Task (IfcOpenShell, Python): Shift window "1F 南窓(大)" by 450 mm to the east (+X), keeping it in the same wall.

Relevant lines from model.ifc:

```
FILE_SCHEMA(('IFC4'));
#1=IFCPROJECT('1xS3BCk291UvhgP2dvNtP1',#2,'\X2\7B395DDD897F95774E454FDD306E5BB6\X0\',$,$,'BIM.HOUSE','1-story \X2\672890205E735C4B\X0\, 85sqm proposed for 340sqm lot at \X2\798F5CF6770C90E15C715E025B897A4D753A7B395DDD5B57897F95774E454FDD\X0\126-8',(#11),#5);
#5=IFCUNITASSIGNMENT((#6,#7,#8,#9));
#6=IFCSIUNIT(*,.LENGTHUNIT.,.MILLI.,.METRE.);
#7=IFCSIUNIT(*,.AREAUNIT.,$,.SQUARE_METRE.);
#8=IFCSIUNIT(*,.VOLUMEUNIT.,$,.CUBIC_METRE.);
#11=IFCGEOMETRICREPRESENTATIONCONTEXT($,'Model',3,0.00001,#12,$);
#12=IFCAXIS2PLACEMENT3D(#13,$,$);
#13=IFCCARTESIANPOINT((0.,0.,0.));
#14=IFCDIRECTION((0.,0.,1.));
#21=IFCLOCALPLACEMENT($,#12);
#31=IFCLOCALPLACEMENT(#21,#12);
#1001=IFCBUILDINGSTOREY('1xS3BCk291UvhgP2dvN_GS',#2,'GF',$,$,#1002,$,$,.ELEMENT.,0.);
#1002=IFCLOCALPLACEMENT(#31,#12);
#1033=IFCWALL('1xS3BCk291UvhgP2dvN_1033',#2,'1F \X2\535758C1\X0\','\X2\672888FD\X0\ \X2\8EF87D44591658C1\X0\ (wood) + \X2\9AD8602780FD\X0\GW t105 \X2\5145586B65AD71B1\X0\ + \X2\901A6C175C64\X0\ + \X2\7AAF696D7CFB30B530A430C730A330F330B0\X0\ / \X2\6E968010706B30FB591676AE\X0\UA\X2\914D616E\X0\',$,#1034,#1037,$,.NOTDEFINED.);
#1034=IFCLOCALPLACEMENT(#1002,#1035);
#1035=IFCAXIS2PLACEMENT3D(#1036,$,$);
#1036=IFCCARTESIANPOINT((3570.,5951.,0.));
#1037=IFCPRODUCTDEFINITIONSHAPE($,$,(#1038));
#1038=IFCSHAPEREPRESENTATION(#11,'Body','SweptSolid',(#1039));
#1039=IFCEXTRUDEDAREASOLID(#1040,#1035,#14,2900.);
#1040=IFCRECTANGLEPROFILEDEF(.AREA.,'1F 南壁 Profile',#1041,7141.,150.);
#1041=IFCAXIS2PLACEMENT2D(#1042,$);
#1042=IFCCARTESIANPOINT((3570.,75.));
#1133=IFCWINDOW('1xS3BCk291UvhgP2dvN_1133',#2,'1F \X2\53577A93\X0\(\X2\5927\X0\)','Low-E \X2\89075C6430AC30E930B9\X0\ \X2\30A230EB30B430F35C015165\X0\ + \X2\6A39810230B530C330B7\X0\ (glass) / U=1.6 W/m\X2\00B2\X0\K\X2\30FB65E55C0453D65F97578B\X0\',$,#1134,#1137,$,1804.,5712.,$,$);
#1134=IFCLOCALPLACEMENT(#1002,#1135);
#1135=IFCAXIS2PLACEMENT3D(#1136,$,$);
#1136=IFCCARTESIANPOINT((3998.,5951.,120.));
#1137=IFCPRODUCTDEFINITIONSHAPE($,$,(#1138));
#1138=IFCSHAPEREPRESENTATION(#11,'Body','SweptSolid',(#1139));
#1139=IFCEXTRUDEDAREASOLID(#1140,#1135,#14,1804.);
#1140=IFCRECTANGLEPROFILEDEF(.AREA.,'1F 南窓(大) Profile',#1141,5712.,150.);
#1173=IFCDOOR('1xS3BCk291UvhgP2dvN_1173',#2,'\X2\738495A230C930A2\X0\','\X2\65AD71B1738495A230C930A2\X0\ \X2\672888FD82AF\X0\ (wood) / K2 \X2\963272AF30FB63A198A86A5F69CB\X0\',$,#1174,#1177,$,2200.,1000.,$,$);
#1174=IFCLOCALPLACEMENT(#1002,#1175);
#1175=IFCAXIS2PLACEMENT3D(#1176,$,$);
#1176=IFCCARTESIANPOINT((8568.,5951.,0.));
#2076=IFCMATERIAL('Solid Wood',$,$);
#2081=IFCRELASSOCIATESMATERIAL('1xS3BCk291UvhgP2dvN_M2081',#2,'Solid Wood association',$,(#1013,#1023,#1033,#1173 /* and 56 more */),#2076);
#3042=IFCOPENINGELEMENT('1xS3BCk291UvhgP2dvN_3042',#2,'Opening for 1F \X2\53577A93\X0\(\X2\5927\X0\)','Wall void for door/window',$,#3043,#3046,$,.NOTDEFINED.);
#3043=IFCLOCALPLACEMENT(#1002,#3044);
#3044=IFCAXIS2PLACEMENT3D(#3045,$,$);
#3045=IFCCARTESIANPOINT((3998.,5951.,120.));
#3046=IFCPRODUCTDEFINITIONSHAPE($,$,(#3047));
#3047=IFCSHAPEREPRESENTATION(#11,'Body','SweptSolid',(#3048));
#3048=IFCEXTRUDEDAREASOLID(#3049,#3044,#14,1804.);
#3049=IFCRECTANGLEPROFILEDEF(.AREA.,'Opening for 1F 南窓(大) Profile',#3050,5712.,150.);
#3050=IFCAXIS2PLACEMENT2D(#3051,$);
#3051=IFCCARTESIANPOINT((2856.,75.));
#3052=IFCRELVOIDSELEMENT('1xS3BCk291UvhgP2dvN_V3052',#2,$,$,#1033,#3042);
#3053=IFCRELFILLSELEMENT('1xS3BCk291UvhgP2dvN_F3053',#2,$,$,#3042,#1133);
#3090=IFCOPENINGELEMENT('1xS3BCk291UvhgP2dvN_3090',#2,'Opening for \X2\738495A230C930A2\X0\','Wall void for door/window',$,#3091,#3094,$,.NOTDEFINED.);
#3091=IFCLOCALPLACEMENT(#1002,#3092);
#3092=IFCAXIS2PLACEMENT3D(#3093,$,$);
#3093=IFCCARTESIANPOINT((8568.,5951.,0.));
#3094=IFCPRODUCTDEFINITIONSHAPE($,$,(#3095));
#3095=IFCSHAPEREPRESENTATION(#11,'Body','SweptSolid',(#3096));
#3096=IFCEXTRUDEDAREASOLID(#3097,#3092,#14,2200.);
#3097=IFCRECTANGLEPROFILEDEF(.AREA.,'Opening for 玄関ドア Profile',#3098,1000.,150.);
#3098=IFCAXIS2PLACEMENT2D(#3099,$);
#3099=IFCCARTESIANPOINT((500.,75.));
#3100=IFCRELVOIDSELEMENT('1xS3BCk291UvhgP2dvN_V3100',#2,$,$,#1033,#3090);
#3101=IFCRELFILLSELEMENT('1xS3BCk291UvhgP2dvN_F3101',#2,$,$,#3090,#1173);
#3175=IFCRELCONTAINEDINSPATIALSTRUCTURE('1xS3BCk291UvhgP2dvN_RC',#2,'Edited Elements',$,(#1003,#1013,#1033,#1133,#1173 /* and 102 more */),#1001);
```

```python
import ifcopenshell
import ifcopenshell.api.geometry
import ifcopenshell.util.placement
import ifcopenshell.util.unit

model = ifcopenshell.open("model.ifc")
unit_scale = ifcopenshell.util.unit.calculate_unit_scale(model)

window = model.by_id(1133)
opening = window.FillsVoids[0].RelatingOpeningElement
wall = opening.VoidsElements[0].RelatingBuildingElement

wall_matrix = ifcopenshell.util.placement.get_local_placement(wall.ObjectPlacement)
shift = wall_matrix[:3, 0] * 0.45 / unit_scale
before = ifcopenshell.util.placement.get_local_placement(window.ObjectPlacement)[:3, 3].copy()

# The window is not placed relative to its opening, so move both.
for product in (opening, window):
    matrix = ifcopenshell.util.placement.get_local_placement(product.ObjectPlacement)
    matrix[:3, 3] += shift
    ifcopenshell.api.geometry.edit_object_placement(model, product=product, matrix=matrix, is_si=False)

after = ifcopenshell.util.placement.get_local_placement(window.ObjectPlacement)[:3, 3]
print("window moved by", (after - before).round(3) + 0.0)

model.write("model_v2.ifc")
```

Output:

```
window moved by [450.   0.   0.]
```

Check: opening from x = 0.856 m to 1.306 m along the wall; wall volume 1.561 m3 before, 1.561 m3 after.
